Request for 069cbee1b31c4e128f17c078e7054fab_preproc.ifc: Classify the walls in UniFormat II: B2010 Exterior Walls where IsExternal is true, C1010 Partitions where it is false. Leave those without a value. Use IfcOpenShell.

First a look at what the model holds.

```python
import ifcopenshell
import ifcopenshell.util.element

model = ifcopenshell.open("069cbee1b31c4e128f17c078e7054fab_preproc.ifc")
print(model.schema)
print("classifications:", [c.Name for c in model.by_type("IfcClassification")])
values = [ifcopenshell.util.element.get_pset(e, "Pset_WallCommon", "IsExternal") for e in model.by_type("IfcWall")]
for value in (True, False, None):
    print("IsExternal", value, values.count(value))
```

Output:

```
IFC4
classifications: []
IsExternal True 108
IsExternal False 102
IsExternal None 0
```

```python
import ifcopenshell
import ifcopenshell.api.classification
import ifcopenshell.util.element

model = ifcopenshell.open("069cbee1b31c4e128f17c078e7054fab_preproc.ifc")

system = ifcopenshell.api.classification.add_classification(model, classification="UniFormat II")

walls = model.by_type("IfcWall")
external = {e: ifcopenshell.util.element.get_pset(e, "Pset_WallCommon", "IsExternal") for e in walls}
for flag, code, name in ((True, "B2010", "Exterior Walls"), (False, "C1010", "Partitions")):
    products = [e for e in walls if external[e] is flag]
    ifcopenshell.api.classification.add_reference(
        model, products=products, classification=system, identification=code, name=name
    )
    print(code, len(products))

model.write("069cbee1b31c4e128f17c078e7054fab_preproc_edited.ifc")
```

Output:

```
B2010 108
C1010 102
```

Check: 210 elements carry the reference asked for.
